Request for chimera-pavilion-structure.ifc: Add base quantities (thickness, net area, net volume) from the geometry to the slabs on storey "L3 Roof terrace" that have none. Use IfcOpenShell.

First a look at what the model holds.

```python
import ifcopenshell
import ifcopenshell.util.element
import ifcopenshell.util.unit

model = ifcopenshell.open("chimera-pavilion-structure.ifc")
print(model.schema)
for unit_type in ("LENGTHUNIT", "AREAUNIT", "VOLUMEUNIT"):
    print(unit_type, ifcopenshell.util.unit.calculate_unit_scale(model, unit_type))
storey = next(s for s in model.by_type("IfcBuildingStorey") if s.Name == "L3 Roof terrace")
slabs = [e for e in ifcopenshell.util.element.get_decomposition(storey) if e.is_a("IfcSlab")]
for e in sorted(slabs, key=lambda e: e.id()):
    print(e.id(), e.is_a(), e.Name, list(ifcopenshell.util.element.get_psets(e, qtos_only=True)), sep=" | ")
```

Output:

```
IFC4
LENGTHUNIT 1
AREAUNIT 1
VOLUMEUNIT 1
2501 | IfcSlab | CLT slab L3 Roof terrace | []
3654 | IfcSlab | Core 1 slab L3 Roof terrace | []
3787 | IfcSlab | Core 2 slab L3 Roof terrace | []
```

```python
import ifcopenshell
import ifcopenshell.api.pset
import ifcopenshell.geom
import ifcopenshell.util.element
import ifcopenshell.util.shape
import ifcopenshell.util.unit

model = ifcopenshell.open("chimera-pavilion-structure.ifc")
unit_scale = ifcopenshell.util.unit.calculate_unit_scale(model)
area_scale = ifcopenshell.util.unit.calculate_unit_scale(model, "AREAUNIT")
volume_scale = ifcopenshell.util.unit.calculate_unit_scale(model, "VOLUMEUNIT")
settings = ifcopenshell.geom.settings()

storey = next(s for s in model.by_type("IfcBuildingStorey") if s.Name == "L3 Roof terrace")
slabs = [e for e in ifcopenshell.util.element.get_decomposition(storey) if e.is_a("IfcSlab")]

for e in sorted(slabs, key=lambda e: e.id()):
    if ifcopenshell.util.element.get_psets(e, qtos_only=True, should_inherit=False):
        continue
    # Geometry comes back in metres, in the element's own axes.
    shape = ifcopenshell.geom.create_shape(settings, e)
    values = {
        "Width": ifcopenshell.util.shape.get_z(shape.geometry) / unit_scale,
        "NetArea": ifcopenshell.util.shape.get_footprint_area(shape.geometry) / area_scale,
        "NetVolume": ifcopenshell.util.shape.get_volume(shape.geometry) / volume_scale,
    }
    qto = ifcopenshell.api.pset.add_qto(model, product=e, name="Qto_SlabBaseQuantities")
    ifcopenshell.api.pset.edit_qto(model, qto=qto, properties=values)
    print(e.id(), {k: round(v, 3) for k, v in values.items()})

model.write("chimera-pavilion-structure_edited.ifc")
```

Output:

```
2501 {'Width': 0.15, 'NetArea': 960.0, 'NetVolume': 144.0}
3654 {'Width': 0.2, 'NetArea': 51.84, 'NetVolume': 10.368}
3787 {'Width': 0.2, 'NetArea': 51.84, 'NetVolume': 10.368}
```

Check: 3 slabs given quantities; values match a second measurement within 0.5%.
